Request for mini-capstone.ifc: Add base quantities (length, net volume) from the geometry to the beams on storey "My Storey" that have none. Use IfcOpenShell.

First a look at what the model holds.

```python
import ifcopenshell
import ifcopenshell.util.element
import ifcopenshell.util.unit

model = ifcopenshell.open("mini-capstone.ifc")
print(model.schema)
for unit_type in ("LENGTHUNIT", "AREAUNIT", "VOLUMEUNIT"):
    print(unit_type, ifcopenshell.util.unit.calculate_unit_scale(model, unit_type))
storey = next(s for s in model.by_type("IfcBuildingStorey") if s.Name == "My Storey")
beams = [e for e in ifcopenshell.util.element.get_decomposition(storey) if e.is_a("IfcBeam")]
for e in sorted(beams, key=lambda e: e.id()):
    print(e.id(), e.is_a(), e.Name, list(ifcopenshell.util.element.get_psets(e, qtos_only=True)), sep=" | ")
```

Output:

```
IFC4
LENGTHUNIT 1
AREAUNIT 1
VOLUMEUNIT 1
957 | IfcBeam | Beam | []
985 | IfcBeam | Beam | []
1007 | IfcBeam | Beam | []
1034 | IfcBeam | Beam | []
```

```python
import ifcopenshell
import ifcopenshell.api.pset
import ifcopenshell.geom
import ifcopenshell.util.element
import ifcopenshell.util.shape
import ifcopenshell.util.unit

model = ifcopenshell.open("mini-capstone.ifc")
unit_scale = ifcopenshell.util.unit.calculate_unit_scale(model)
volume_scale = ifcopenshell.util.unit.calculate_unit_scale(model, "VOLUMEUNIT")
settings = ifcopenshell.geom.settings()

storey = next(s for s in model.by_type("IfcBuildingStorey") if s.Name == "My Storey")
beams = [e for e in ifcopenshell.util.element.get_decomposition(storey) if e.is_a("IfcBeam")]

for e in sorted(beams, key=lambda e: e.id()):
    if ifcopenshell.util.element.get_psets(e, qtos_only=True, should_inherit=False):
        continue
    # Geometry comes back in metres, in the element's own axes.
    shape = ifcopenshell.geom.create_shape(settings, e)
    values = {
        "Length": ifcopenshell.util.shape.get_max_xyz(shape.geometry) / unit_scale,
        "NetVolume": ifcopenshell.util.shape.get_volume(shape.geometry) / volume_scale,
    }
    qto = ifcopenshell.api.pset.add_qto(model, product=e, name="Qto_BeamBaseQuantities")
    ifcopenshell.api.pset.edit_qto(model, qto=qto, properties=values)
    print(e.id(), {k: round(v, 3) for k, v in values.items()})

model.write("mini-capstone_edited.ifc")
```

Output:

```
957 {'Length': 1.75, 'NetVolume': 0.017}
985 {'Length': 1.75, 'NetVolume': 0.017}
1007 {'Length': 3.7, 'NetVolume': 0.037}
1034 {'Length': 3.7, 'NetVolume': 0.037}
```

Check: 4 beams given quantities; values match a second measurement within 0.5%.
